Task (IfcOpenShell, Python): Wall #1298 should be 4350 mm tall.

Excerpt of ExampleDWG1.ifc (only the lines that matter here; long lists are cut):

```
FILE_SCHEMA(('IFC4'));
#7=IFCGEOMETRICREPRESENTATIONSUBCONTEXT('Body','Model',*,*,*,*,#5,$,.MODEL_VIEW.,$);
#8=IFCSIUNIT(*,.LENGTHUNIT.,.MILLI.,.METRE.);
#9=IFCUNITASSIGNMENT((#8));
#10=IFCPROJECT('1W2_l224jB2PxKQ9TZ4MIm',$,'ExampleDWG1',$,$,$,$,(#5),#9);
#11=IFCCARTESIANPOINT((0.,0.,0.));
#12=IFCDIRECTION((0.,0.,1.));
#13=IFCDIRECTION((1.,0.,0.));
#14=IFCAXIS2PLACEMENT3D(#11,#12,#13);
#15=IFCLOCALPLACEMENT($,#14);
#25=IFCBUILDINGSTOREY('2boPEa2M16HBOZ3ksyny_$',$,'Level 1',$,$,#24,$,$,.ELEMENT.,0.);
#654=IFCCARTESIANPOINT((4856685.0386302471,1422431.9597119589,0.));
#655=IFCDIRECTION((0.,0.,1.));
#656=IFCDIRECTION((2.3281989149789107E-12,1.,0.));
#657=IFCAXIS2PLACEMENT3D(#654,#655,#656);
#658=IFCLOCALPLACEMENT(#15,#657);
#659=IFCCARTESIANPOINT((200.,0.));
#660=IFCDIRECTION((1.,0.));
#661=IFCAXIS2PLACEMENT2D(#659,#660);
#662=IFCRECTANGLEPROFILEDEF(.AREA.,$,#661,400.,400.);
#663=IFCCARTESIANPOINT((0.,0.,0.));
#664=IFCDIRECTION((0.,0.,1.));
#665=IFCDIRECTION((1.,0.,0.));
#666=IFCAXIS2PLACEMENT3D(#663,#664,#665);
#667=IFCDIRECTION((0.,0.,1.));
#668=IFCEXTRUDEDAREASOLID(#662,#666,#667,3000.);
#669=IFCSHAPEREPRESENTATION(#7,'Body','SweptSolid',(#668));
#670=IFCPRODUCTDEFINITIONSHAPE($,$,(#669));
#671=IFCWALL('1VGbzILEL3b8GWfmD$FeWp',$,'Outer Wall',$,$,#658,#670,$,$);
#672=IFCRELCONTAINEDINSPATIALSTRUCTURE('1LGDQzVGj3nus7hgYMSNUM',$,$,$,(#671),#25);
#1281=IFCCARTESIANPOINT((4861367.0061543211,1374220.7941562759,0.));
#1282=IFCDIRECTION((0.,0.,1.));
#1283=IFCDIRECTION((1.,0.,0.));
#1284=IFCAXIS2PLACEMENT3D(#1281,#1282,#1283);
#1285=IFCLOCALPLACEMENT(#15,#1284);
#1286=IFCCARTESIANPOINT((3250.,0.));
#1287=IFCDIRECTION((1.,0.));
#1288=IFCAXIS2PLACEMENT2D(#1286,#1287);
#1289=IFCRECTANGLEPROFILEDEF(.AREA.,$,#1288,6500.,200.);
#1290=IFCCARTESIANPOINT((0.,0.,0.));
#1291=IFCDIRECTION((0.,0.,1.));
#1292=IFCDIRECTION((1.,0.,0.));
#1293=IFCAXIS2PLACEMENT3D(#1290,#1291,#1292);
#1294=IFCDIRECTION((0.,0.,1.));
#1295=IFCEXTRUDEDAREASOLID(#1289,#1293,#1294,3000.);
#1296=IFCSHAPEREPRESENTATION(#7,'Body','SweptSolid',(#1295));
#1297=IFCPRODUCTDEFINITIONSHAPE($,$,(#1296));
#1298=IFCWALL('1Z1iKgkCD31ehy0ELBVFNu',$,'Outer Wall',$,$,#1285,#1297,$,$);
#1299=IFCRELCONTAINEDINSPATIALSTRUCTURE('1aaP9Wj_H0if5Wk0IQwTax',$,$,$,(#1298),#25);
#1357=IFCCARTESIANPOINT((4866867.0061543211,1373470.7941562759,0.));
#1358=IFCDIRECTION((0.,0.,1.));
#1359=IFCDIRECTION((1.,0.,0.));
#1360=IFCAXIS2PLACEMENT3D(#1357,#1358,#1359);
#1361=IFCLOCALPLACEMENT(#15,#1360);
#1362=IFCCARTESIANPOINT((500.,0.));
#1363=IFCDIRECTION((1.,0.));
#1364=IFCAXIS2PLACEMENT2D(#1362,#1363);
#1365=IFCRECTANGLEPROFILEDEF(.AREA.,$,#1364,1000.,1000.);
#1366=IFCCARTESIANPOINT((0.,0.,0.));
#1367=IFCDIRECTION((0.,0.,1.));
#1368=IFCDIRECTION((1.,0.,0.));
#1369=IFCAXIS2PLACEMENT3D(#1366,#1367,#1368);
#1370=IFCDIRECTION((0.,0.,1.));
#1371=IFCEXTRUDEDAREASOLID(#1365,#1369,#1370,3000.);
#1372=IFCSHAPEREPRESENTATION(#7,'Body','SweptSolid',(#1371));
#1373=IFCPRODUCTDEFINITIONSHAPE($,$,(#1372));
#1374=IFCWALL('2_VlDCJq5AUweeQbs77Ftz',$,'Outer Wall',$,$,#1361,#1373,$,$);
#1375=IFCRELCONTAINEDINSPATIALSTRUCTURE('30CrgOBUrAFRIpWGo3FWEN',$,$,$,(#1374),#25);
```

```python
import ifcopenshell
import ifcopenshell.geom
import ifcopenshell.util.representation
import ifcopenshell.util.shape

model = ifcopenshell.open("ExampleDWG1.ifc")
settings = ifcopenshell.geom.settings()


def volume(element):
    """Net volume in cubic metres, openings subtracted."""
    shape = ifcopenshell.geom.create_shape(settings, element)
    return ifcopenshell.util.shape.get_volume(shape.geometry)


wall = model.by_guid("1Z1iKgkCD31ehy0ELBVFNu")
before = volume(wall)

body = ifcopenshell.util.representation.get_representation(wall, "Model", "Body")
solid = body.Items[0]
old_height = solid.Depth
solid.Depth = 4350.0
after = volume(wall)

print(f"height {old_height:g} -> {solid.Depth:g}, volume {before:.3f} -> {after:.3f} m3")

model.write("ExampleDWG1_updated.ifc")
```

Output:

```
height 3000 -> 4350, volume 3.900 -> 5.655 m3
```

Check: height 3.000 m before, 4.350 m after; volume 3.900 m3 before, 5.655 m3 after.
